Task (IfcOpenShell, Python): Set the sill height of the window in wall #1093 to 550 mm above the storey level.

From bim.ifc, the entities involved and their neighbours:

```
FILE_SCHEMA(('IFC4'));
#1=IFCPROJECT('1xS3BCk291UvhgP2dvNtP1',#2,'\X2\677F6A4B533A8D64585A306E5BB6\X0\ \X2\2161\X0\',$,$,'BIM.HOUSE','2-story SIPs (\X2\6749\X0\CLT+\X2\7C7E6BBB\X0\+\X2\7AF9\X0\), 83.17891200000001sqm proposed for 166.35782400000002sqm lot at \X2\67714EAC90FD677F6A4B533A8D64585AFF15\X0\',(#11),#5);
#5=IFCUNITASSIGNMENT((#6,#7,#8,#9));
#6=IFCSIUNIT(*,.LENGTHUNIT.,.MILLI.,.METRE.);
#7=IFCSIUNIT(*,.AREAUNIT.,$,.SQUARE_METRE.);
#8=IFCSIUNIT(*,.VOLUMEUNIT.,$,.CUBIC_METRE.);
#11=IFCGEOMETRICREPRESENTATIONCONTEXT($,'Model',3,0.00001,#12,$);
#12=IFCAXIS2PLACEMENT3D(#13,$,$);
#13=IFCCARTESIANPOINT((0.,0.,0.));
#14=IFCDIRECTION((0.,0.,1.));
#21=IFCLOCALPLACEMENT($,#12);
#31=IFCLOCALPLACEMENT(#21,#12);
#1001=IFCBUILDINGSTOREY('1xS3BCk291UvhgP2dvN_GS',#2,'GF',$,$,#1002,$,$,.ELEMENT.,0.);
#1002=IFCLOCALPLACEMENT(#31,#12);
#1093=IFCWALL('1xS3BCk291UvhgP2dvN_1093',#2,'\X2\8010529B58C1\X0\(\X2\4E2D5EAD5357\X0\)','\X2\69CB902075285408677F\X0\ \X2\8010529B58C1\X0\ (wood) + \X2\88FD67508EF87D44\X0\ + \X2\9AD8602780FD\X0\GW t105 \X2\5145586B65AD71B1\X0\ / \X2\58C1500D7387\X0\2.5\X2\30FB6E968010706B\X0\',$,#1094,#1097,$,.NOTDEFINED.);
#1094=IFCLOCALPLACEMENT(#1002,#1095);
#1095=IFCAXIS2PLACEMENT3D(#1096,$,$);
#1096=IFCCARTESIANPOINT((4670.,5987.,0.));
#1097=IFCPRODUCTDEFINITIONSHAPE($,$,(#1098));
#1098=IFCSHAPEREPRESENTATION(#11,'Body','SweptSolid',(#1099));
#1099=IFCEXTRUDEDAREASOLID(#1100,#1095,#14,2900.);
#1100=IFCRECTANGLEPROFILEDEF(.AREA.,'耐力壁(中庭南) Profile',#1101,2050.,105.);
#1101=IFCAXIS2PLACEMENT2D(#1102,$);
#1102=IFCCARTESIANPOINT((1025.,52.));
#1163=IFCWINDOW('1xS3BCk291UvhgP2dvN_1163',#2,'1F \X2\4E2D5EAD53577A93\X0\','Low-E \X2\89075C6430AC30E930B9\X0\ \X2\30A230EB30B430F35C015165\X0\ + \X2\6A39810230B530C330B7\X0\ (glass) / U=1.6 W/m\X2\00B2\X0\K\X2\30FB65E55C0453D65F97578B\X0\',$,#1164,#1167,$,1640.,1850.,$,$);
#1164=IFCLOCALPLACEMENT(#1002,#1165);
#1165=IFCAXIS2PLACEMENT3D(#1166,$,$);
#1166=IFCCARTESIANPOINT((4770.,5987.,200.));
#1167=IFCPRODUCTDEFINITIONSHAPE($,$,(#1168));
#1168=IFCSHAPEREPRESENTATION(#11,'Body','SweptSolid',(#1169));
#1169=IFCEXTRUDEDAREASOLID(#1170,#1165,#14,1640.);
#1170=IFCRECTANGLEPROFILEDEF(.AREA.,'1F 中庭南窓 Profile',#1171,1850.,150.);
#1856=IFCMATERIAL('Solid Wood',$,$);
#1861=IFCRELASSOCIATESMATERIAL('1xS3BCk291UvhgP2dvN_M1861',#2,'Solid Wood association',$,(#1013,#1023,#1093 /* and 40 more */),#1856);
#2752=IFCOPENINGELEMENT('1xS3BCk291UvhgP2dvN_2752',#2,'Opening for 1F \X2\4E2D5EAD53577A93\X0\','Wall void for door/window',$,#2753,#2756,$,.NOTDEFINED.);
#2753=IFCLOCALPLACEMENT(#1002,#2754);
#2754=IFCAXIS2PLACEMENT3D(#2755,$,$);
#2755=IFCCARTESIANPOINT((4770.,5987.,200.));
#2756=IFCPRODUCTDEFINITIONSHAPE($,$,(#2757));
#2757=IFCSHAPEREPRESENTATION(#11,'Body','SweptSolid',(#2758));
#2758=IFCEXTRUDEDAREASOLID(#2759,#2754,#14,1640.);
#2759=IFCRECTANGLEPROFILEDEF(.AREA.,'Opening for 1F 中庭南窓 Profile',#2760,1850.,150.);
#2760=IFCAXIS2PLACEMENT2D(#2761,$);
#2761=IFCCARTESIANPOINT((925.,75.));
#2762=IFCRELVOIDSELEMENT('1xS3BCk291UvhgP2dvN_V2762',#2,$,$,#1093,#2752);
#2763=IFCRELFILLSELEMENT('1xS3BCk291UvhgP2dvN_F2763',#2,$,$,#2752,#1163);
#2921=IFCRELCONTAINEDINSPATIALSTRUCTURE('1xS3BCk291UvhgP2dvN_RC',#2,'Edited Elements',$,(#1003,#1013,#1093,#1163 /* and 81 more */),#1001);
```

```python
import numpy as np
import ifcopenshell
import ifcopenshell.api.geometry
import ifcopenshell.geom
import ifcopenshell.util.element
import ifcopenshell.util.placement
import ifcopenshell.util.shape
import ifcopenshell.util.unit

model = ifcopenshell.open("bim.ifc")
unit_scale = ifcopenshell.util.unit.calculate_unit_scale(model)

window = model.by_guid("1xS3BCk291UvhgP2dvN_1163")
opening = window.FillsVoids[0].RelatingOpeningElement
storey = ifcopenshell.util.element.get_container(window, ifc_class="IfcBuildingStorey")
level = ifcopenshell.util.placement.get_local_placement(storey.ObjectPlacement)[2, 3]

# The opening's origin need not be at the sill, so measure its lowest point.
shape = ifcopenshell.geom.create_shape(ifcopenshell.geom.settings(), opening)
bottom = ifcopenshell.util.shape.get_shape_bottom_elevation(shape, shape.geometry) / unit_scale
dz = level + 0.55 / unit_scale - bottom

shift = np.array([0.0, 0.0, dz])
# The window is not placed relative to its opening, so move both.
for product in (opening, window):
    matrix = ifcopenshell.util.placement.get_local_placement(product.ObjectPlacement)
    matrix[:3, 3] += shift
    ifcopenshell.api.geometry.edit_object_placement(model, product=product, matrix=matrix, is_si=False)

print(f"moved by {dz * unit_scale:+.3f} m")

model.write("bim-out.ifc")
```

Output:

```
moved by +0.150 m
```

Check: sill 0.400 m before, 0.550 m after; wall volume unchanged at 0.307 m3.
